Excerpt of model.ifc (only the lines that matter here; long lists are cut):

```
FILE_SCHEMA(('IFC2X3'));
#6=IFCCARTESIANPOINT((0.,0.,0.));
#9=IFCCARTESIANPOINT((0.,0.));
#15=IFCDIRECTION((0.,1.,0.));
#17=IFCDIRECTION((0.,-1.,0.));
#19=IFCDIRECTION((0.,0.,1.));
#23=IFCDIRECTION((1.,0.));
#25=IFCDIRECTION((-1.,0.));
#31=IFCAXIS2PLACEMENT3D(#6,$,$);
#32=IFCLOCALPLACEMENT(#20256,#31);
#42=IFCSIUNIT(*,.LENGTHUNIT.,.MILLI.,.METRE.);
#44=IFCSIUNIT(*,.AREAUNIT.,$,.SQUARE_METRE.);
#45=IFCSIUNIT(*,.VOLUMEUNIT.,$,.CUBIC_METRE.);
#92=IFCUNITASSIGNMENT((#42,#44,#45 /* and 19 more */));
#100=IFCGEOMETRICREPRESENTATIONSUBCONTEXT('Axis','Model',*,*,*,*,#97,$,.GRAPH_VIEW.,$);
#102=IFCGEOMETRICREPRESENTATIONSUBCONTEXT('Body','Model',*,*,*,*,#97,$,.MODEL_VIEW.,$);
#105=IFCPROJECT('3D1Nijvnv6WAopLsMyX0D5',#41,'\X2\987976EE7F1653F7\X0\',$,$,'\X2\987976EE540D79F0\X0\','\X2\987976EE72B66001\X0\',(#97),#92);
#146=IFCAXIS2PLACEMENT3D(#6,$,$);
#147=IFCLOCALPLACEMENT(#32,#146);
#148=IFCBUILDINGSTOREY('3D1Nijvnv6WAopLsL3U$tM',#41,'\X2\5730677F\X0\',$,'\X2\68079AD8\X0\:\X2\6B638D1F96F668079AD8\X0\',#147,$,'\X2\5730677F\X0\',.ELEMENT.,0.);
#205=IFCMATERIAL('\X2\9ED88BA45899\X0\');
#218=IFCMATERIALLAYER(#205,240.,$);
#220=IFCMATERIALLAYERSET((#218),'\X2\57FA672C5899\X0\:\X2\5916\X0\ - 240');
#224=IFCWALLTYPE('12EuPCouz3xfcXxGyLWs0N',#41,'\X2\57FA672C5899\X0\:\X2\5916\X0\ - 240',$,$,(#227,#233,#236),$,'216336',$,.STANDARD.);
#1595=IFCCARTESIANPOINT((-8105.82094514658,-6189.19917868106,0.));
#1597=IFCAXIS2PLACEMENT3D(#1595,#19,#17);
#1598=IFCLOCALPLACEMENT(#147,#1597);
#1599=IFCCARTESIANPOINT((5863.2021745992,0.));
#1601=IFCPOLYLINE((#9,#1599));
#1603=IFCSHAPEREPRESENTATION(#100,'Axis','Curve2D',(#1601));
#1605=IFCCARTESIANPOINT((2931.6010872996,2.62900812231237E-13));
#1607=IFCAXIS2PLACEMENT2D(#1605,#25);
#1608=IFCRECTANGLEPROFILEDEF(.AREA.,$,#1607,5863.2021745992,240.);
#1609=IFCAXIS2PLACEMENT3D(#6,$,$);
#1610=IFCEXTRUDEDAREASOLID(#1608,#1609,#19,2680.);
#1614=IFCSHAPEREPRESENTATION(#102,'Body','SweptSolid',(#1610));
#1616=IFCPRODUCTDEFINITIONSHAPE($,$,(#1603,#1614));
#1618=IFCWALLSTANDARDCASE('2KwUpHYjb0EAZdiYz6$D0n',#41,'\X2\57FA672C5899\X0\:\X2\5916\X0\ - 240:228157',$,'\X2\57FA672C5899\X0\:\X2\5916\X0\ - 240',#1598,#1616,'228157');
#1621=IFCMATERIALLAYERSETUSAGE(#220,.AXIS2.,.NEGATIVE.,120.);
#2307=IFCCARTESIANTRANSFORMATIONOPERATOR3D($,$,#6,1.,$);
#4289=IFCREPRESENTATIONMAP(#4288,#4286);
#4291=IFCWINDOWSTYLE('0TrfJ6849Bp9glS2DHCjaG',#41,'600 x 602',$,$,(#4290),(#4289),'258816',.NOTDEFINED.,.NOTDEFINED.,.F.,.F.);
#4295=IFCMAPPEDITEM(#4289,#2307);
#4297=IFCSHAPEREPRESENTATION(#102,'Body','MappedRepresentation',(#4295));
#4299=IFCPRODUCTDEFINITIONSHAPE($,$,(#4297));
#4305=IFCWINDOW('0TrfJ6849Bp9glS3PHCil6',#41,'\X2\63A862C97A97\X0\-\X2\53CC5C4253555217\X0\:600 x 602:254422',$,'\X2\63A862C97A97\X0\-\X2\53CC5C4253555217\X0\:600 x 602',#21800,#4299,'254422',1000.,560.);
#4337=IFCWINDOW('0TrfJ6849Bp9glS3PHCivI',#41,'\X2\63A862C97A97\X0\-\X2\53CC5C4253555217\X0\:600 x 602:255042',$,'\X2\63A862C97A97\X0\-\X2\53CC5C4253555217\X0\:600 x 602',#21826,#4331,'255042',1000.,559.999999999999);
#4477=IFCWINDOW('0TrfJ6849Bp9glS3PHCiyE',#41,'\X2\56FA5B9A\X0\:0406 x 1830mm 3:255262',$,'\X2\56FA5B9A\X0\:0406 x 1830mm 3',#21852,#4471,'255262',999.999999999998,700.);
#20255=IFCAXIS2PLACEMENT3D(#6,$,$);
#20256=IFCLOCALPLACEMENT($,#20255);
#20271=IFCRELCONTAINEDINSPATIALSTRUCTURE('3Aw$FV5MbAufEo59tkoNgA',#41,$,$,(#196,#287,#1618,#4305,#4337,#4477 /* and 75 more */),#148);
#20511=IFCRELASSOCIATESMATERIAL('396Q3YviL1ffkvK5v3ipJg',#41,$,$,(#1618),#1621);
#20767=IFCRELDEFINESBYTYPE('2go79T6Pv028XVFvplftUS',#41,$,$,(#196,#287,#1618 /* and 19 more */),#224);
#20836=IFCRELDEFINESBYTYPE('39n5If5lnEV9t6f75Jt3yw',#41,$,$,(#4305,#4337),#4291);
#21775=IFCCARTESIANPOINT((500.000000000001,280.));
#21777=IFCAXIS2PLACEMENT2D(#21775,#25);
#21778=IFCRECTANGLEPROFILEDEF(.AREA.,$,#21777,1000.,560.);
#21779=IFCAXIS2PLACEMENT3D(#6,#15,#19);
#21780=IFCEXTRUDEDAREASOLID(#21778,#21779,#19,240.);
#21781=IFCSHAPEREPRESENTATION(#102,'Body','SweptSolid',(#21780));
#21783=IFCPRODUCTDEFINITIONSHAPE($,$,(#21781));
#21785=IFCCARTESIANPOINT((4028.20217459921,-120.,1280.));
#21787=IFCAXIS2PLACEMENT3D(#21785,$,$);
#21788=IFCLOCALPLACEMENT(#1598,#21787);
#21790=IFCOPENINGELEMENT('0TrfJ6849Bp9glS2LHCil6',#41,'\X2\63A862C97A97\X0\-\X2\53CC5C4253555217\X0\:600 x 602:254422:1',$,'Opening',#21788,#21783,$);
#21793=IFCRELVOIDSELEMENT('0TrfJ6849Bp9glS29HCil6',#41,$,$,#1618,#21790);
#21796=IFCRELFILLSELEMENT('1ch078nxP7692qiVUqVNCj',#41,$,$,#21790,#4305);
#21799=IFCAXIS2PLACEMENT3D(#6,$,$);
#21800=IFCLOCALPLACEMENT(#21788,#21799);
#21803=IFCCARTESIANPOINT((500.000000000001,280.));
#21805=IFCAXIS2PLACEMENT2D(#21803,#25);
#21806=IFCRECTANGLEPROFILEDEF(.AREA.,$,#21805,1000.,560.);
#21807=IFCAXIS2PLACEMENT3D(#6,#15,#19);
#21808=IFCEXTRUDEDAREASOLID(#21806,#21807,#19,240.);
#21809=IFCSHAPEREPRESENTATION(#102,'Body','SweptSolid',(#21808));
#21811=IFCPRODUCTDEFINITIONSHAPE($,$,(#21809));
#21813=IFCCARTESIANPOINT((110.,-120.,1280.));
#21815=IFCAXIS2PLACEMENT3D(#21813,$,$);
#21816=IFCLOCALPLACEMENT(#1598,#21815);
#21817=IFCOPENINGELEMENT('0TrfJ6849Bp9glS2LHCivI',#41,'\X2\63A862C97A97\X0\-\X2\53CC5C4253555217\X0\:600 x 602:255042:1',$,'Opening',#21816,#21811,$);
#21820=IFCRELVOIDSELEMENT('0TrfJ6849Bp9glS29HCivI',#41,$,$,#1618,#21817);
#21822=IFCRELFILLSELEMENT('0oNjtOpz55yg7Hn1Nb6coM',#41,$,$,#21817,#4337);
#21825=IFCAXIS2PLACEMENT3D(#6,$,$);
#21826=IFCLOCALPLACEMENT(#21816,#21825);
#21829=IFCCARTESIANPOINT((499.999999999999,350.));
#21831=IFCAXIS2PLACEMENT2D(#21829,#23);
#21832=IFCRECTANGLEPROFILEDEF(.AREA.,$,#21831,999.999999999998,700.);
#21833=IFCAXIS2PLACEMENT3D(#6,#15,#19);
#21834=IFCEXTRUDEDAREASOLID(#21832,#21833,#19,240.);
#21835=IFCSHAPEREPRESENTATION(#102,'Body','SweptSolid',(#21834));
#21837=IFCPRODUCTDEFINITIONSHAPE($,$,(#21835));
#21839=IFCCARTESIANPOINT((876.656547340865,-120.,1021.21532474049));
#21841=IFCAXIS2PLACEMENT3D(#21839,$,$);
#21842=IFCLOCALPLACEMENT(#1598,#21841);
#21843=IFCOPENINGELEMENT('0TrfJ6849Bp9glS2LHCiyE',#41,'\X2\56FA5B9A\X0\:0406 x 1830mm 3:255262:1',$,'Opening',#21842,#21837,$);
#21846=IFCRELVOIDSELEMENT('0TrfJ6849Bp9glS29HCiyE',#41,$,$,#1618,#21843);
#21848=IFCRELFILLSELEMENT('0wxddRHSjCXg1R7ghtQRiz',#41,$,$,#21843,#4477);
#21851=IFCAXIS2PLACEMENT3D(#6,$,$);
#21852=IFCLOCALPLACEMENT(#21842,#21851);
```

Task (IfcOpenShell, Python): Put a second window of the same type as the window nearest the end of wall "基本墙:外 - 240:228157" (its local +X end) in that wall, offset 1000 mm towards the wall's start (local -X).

```python
import ifcopenshell
import ifcopenshell.api.feature
import ifcopenshell.api.geometry
import ifcopenshell.api.root
import ifcopenshell.geom
import ifcopenshell.util.element
import ifcopenshell.util.placement
import ifcopenshell.util.shape

model = ifcopenshell.open("model.ifc")
settings = ifcopenshell.geom.settings()


def volume(element):
    """Net volume in cubic metres, openings subtracted."""
    shape = ifcopenshell.geom.create_shape(settings, element)
    return ifcopenshell.util.shape.get_volume(shape.geometry)


def reuse_history(source, copy):
    """copy_class also copies each property set's owner history, people and application; keep the originals."""
    for rel in copy.IsDefinedBy:
        if rel.is_a("IfcRelDefinesByProperties") and (history := rel.RelatingPropertyDefinition.OwnerHistory):
            rel.RelatingPropertyDefinition.OwnerHistory = source.OwnerHistory
            ifcopenshell.util.element.remove_deep2(model, history)


window = model.by_id(4305)
opening = window.FillsVoids[0].RelatingOpeningElement
wall = opening.VoidsElements[0].RelatingBuildingElement
before = volume(wall)
shift = ifcopenshell.util.placement.get_local_placement(wall.ObjectPlacement)[:3, 0] * -1000.0

# copy_class copies the void relationship, type, container and properties, but no geometry.
new_opening = ifcopenshell.api.root.copy_class(model, product=opening)
new_opening.Representation = ifcopenshell.util.element.copy_deep(
    model, opening.Representation, exclude=["IfcGeometricRepresentationContext", "IfcRepresentationMap"]
)
new_opening.Name = "推拉窗-双层单列:600 x 602"
new_window = ifcopenshell.api.root.copy_class(model, product=window)
new_window.Representation = ifcopenshell.util.element.copy_deep(
    model, window.Representation, exclude=["IfcGeometricRepresentationContext", "IfcRepresentationMap"]
)
new_window.Name = "推拉窗-双层单列:600 x 602"
new_window.Tag = None
reuse_history(window, new_window)
fills = ifcopenshell.api.feature.add_filling(model, opening=new_opening, element=new_window)
fills.OwnerHistory = new_window.OwnerHistory  # required in IFC2X3

for old, new in ((opening, new_opening), (window, new_window)):
    matrix = ifcopenshell.util.placement.get_local_placement(old.ObjectPlacement)
    matrix[:3, 3] += shift
    ifcopenshell.api.geometry.edit_object_placement(model, product=new, matrix=matrix, is_si=False)

after = volume(wall)

print(f"wall volume {before:.3f} -> {after:.3f} m3")

model.write("model_edited.ifc")
```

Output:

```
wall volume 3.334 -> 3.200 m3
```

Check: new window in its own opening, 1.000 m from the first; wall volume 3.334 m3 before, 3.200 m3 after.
